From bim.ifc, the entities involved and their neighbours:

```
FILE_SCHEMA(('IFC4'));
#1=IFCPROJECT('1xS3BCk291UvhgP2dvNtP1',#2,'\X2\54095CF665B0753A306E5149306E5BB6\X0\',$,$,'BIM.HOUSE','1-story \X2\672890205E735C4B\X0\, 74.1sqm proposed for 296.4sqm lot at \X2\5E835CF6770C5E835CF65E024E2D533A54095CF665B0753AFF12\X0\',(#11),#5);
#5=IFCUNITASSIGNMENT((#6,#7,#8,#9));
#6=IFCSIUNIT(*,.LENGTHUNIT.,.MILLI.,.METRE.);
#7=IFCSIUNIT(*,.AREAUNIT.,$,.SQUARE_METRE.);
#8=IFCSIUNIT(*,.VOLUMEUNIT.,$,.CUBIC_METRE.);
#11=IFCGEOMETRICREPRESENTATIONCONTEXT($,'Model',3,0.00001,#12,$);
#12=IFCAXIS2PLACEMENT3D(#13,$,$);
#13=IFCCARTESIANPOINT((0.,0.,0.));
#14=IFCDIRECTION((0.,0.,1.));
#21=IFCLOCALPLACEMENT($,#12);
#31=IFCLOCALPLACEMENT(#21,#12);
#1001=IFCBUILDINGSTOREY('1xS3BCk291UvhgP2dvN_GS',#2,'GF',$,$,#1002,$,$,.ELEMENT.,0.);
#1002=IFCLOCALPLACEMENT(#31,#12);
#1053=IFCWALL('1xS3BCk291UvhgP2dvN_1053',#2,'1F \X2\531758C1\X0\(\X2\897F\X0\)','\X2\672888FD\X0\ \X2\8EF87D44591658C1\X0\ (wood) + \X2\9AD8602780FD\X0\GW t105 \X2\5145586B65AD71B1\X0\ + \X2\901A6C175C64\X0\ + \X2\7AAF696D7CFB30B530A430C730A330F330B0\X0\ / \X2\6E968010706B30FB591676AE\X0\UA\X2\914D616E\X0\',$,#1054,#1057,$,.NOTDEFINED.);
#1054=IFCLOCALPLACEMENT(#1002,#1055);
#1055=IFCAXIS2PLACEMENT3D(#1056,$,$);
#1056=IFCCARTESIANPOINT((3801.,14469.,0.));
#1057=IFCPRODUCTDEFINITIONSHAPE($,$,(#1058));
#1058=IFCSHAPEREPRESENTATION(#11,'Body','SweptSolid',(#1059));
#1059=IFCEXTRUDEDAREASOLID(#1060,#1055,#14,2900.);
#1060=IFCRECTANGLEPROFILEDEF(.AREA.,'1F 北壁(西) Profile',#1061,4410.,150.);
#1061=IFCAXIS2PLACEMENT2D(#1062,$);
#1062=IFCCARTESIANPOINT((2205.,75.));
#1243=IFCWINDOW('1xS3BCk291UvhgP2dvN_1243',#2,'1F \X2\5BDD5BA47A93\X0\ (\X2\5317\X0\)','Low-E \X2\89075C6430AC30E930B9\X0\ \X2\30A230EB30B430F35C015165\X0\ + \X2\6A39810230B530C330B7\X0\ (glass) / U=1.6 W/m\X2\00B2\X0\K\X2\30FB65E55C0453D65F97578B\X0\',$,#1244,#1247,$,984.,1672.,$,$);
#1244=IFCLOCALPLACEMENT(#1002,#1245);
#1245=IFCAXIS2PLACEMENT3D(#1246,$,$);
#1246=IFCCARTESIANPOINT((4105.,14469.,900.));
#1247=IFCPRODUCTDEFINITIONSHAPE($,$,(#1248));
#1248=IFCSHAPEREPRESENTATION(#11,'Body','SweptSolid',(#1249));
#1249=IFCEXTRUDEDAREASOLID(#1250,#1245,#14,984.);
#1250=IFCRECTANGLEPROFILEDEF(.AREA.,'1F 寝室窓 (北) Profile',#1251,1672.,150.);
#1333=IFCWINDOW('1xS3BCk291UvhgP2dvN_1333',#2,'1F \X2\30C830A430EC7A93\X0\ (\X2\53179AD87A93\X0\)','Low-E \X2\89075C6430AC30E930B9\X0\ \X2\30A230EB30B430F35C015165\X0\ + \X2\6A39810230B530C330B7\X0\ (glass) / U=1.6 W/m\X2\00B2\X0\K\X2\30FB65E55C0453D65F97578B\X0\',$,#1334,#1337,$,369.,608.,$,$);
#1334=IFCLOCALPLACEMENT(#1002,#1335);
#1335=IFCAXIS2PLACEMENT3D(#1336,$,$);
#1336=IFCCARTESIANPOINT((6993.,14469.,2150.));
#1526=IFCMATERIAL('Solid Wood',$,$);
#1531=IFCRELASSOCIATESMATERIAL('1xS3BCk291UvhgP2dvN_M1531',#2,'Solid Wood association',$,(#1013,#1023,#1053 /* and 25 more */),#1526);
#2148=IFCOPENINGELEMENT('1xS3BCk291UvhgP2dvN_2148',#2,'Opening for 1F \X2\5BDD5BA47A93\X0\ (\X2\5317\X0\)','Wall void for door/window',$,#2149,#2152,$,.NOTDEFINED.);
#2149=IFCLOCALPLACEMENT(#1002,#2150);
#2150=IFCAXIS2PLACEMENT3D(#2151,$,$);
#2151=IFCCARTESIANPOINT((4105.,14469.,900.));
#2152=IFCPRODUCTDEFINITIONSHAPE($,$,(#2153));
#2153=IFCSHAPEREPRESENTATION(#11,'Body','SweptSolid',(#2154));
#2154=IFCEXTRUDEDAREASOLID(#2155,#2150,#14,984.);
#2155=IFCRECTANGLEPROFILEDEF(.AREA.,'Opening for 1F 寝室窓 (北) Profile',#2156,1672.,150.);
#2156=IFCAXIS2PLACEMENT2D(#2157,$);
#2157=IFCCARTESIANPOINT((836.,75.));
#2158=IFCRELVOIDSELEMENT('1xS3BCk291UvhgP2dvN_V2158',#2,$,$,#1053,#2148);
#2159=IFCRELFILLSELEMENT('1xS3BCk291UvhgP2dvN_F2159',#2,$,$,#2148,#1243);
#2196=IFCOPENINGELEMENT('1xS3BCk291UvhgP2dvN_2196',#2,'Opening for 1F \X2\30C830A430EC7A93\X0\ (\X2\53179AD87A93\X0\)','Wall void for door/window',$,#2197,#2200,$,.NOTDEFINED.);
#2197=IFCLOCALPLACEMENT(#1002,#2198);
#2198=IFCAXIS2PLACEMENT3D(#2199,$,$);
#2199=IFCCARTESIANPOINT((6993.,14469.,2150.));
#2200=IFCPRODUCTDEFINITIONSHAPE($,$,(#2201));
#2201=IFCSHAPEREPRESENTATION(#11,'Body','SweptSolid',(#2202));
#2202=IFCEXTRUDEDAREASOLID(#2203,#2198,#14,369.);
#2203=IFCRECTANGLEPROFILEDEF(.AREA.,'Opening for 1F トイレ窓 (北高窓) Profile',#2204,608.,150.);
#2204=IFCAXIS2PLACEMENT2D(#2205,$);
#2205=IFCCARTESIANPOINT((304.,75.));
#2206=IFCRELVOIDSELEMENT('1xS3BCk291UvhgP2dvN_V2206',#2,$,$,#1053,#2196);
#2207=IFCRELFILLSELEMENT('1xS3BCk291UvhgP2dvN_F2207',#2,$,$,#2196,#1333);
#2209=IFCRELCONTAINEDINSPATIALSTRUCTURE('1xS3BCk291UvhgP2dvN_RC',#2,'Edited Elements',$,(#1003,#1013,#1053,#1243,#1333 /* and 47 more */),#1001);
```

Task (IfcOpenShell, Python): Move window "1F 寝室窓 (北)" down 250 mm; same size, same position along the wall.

```python
import numpy as np
import ifcopenshell
import ifcopenshell.api.geometry
import ifcopenshell.util.placement
import ifcopenshell.util.unit

model = ifcopenshell.open("bim.ifc")
unit_scale = ifcopenshell.util.unit.calculate_unit_scale(model)

window = model.by_guid("1xS3BCk291UvhgP2dvN_1243")
opening = window.FillsVoids[0].RelatingOpeningElement
dz = -0.25 / unit_scale

shift = np.array([0.0, 0.0, dz])
# The window is not placed relative to its opening, so move both.
for product in (opening, window):
    matrix = ifcopenshell.util.placement.get_local_placement(product.ObjectPlacement)
    matrix[:3, 3] += shift
    ifcopenshell.api.geometry.edit_object_placement(model, product=product, matrix=matrix, is_si=False)

print(f"moved by {dz * unit_scale:+.3f} m")

model.write("bim_v2.ifc")
```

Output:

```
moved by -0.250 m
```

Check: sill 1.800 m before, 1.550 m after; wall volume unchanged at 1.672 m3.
